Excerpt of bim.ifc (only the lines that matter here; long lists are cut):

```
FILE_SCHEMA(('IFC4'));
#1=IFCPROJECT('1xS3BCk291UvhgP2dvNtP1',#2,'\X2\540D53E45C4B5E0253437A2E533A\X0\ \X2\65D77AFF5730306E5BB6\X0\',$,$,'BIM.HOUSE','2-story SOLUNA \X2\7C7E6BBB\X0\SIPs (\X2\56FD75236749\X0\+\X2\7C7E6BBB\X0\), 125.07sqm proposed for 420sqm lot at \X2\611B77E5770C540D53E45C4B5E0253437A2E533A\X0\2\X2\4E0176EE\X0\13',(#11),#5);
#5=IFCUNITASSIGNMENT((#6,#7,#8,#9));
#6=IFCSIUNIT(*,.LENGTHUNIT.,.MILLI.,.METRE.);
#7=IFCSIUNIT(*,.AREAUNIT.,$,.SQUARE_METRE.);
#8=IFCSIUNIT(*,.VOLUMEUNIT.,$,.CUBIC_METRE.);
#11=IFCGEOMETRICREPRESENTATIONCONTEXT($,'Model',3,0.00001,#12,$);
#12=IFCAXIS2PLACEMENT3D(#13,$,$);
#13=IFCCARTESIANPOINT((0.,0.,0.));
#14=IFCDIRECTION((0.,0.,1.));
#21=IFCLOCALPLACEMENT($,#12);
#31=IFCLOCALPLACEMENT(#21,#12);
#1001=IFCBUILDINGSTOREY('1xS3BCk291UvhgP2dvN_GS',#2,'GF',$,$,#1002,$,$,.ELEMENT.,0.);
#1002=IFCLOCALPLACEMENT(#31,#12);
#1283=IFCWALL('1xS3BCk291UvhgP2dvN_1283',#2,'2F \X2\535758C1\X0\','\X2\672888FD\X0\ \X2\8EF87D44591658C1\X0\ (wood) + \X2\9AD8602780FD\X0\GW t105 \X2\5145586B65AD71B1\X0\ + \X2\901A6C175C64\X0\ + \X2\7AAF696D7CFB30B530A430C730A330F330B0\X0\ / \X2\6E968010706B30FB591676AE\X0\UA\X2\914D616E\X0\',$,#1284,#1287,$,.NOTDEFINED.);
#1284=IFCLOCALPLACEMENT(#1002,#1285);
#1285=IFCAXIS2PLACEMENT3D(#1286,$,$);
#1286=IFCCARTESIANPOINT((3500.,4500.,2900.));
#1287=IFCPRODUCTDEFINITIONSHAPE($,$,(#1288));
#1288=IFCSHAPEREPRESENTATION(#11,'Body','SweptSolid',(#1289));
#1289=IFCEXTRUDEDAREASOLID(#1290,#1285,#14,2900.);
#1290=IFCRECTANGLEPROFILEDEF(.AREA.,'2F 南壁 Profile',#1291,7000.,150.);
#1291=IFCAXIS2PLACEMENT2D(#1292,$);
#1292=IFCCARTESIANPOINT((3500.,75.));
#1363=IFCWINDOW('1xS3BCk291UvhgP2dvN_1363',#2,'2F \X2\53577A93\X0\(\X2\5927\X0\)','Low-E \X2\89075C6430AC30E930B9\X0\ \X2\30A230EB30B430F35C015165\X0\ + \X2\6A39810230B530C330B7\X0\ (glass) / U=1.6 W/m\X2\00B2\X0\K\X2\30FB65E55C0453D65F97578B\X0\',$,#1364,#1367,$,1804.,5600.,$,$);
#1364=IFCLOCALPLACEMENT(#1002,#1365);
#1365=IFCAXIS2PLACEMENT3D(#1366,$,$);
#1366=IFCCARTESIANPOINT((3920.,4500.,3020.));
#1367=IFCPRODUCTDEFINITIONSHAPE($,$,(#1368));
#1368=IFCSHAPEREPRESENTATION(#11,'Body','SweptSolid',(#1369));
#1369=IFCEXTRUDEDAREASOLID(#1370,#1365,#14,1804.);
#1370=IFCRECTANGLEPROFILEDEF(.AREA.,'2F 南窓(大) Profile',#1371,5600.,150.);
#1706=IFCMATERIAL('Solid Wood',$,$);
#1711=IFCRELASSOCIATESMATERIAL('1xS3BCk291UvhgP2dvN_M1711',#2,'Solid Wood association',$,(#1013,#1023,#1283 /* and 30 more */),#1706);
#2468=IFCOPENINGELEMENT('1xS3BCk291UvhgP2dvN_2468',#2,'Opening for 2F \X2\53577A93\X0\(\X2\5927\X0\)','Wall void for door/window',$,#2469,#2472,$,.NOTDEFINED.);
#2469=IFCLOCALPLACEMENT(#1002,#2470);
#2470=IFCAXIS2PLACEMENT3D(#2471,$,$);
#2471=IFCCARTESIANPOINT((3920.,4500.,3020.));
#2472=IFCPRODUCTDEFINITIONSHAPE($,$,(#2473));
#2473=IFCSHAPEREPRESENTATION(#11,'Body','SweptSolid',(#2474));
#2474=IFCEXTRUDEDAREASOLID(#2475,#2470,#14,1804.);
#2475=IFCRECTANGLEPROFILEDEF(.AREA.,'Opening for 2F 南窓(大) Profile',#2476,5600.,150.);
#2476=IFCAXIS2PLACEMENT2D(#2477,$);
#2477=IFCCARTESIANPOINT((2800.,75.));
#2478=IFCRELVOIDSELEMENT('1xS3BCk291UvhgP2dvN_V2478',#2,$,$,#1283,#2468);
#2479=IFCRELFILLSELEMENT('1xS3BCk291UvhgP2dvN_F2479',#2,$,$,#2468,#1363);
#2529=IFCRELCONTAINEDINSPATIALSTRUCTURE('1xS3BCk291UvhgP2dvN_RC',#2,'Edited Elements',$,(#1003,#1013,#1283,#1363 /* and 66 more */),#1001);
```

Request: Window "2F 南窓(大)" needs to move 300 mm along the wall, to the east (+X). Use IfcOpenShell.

```python
import ifcopenshell
import ifcopenshell.api.geometry
import ifcopenshell.util.placement

model = ifcopenshell.open("bim.ifc")

window = model.by_guid("1xS3BCk291UvhgP2dvN_1363")
opening = window.FillsVoids[0].RelatingOpeningElement
wall = opening.VoidsElements[0].RelatingBuildingElement

wall_matrix = ifcopenshell.util.placement.get_local_placement(wall.ObjectPlacement)
shift = wall_matrix[:3, 0] * 300.0
before = ifcopenshell.util.placement.get_local_placement(window.ObjectPlacement)[:3, 3].copy()

# The window is not placed relative to its opening, so move both.
for product in (opening, window):
    matrix = ifcopenshell.util.placement.get_local_placement(product.ObjectPlacement)
    matrix[:3, 3] += shift
    ifcopenshell.api.geometry.edit_object_placement(model, product=product, matrix=matrix, is_si=False)

after = ifcopenshell.util.placement.get_local_placement(window.ObjectPlacement)[:3, 3]
print("window moved by", (after - before).round(3) + 0.0)

model.write("bim-out.ifc")
```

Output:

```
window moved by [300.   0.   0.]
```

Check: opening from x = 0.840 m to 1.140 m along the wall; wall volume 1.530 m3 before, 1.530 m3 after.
